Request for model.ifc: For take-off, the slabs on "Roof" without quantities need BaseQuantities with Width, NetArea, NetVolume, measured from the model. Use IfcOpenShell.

First a look at what the model holds.

```python
import ifcopenshell
import ifcopenshell.util.element
import ifcopenshell.util.unit

model = ifcopenshell.open("model.ifc")
print(model.schema)
for unit_type in ("LENGTHUNIT", "AREAUNIT", "VOLUMEUNIT"):
    print(unit_type, ifcopenshell.util.unit.calculate_unit_scale(model, unit_type))
storey = next(s for s in model.by_type("IfcBuildingStorey") if s.Name == "Roof")
slabs = [e for e in ifcopenshell.util.element.get_decomposition(storey) if e.is_a("IfcSlab")]
for e in sorted(slabs, key=lambda e: e.id()):
    print(e.id(), e.is_a(), e.Name, list(ifcopenshell.util.element.get_psets(e, qtos_only=True)), sep=" | ")
```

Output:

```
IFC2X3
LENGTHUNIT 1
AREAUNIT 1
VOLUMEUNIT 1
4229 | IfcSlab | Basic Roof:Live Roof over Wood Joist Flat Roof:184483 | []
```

```python
import ifcopenshell
import ifcopenshell.api.pset
import ifcopenshell.geom
import ifcopenshell.util.element
import ifcopenshell.util.shape
import ifcopenshell.util.unit

model = ifcopenshell.open("model.ifc")
unit_scale = ifcopenshell.util.unit.calculate_unit_scale(model)
area_scale = ifcopenshell.util.unit.calculate_unit_scale(model, "AREAUNIT")
volume_scale = ifcopenshell.util.unit.calculate_unit_scale(model, "VOLUMEUNIT")
settings = ifcopenshell.geom.settings()

storey = next(s for s in model.by_type("IfcBuildingStorey") if s.Name == "Roof")
slabs = [e for e in ifcopenshell.util.element.get_decomposition(storey) if e.is_a("IfcSlab")]

for e in sorted(slabs, key=lambda e: e.id()):
    if ifcopenshell.util.element.get_psets(e, qtos_only=True, should_inherit=False):
        continue
    # Geometry comes back in metres, in the element's own axes.
    shape = ifcopenshell.geom.create_shape(settings, e)
    values = {
        "Width": ifcopenshell.util.shape.get_z(shape.geometry) / unit_scale,
        "NetArea": ifcopenshell.util.shape.get_footprint_area(shape.geometry) / area_scale,
        "NetVolume": ifcopenshell.util.shape.get_volume(shape.geometry) / volume_scale,
    }
    qto = ifcopenshell.api.pset.add_qto(model, product=e, name="BaseQuantities")
    ifcopenshell.api.pset.edit_qto(model, qto=qto, properties=values)
    print(e.id(), {k: round(v, 3) for k, v in values.items()})

model.write("model_rev.ifc")
```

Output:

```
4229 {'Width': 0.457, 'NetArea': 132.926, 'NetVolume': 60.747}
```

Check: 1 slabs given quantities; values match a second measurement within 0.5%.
